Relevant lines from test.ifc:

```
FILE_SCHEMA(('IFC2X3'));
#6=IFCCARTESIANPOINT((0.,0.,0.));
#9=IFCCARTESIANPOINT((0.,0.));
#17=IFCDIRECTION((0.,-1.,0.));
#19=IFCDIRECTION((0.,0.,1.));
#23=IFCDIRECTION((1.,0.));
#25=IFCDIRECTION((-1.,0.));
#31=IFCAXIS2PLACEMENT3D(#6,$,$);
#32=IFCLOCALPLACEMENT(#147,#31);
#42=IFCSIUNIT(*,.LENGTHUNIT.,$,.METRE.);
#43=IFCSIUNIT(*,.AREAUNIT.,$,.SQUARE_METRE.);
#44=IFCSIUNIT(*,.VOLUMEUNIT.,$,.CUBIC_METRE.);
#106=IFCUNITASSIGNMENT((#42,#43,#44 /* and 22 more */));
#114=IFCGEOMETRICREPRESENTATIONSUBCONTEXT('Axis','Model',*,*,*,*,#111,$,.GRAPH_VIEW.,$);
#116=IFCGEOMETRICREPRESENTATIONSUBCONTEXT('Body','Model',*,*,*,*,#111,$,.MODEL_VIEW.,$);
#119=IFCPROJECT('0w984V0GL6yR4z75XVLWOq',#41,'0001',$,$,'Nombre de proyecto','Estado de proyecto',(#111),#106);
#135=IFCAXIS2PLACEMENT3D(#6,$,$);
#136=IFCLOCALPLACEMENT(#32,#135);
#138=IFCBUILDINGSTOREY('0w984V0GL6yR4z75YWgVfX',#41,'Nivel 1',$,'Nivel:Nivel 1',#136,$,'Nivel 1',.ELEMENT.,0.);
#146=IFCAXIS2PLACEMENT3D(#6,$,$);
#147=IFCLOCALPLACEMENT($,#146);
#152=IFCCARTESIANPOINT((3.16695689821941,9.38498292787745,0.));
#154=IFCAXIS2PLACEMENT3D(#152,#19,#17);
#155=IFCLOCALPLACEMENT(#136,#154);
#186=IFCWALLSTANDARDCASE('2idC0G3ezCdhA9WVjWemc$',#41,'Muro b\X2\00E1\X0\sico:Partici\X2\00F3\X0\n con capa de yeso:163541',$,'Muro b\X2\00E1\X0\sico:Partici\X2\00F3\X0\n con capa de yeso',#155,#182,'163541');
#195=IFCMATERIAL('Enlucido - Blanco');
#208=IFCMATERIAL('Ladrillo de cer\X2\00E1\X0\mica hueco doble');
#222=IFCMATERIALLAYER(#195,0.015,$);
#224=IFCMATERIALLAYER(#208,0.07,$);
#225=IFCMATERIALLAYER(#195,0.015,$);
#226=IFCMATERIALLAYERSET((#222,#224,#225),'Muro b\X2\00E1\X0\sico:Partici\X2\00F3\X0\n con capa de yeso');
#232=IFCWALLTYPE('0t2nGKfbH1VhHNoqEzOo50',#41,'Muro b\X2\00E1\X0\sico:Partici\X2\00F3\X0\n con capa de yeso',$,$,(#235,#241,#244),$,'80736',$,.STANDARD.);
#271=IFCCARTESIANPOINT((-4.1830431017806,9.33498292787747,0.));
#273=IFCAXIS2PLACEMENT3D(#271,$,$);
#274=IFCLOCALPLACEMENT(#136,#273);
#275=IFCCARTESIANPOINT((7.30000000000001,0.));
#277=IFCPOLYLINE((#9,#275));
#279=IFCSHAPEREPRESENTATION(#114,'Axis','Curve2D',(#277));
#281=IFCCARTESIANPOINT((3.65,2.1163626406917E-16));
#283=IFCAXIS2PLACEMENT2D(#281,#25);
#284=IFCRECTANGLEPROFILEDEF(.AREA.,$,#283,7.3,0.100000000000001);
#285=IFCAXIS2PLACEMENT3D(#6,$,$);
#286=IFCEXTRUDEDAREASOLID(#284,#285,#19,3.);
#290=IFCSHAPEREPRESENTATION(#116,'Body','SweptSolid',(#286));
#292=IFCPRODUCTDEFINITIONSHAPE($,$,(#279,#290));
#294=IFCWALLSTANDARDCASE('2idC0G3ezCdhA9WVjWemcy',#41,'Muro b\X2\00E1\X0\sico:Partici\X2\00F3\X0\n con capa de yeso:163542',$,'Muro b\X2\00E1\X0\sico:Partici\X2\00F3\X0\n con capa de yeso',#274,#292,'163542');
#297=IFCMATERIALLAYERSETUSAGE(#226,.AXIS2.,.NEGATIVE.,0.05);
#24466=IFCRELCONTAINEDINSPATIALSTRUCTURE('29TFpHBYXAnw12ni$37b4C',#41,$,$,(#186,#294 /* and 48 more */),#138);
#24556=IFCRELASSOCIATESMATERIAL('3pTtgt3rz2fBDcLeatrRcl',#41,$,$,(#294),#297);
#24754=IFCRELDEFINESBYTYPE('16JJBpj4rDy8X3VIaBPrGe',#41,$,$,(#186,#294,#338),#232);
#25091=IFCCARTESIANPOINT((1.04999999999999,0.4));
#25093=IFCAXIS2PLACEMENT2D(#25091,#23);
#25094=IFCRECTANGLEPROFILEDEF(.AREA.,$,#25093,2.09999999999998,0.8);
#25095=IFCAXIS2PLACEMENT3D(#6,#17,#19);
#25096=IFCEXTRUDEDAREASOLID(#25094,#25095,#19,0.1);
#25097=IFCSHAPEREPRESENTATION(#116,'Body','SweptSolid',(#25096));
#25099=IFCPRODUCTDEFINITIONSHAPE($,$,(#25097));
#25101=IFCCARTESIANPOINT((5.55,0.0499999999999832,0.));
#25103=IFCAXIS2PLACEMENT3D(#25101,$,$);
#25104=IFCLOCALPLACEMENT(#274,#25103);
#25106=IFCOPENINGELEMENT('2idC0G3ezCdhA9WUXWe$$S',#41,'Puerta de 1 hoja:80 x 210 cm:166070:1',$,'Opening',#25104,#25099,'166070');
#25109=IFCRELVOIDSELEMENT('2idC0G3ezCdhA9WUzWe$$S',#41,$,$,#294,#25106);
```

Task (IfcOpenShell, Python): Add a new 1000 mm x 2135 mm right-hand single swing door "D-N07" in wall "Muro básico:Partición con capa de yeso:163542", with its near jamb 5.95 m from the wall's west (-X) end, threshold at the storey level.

```python
import numpy as np
import ifcopenshell
import ifcopenshell.api.feature
import ifcopenshell.api.geometry
import ifcopenshell.api.root
import ifcopenshell.api.spatial
import ifcopenshell.api.type
import ifcopenshell.geom
import ifcopenshell.util.element
import ifcopenshell.util.placement
import ifcopenshell.util.representation
import ifcopenshell.util.shape
import ifcopenshell.util.unit

model = ifcopenshell.open("test.ifc")
unit_scale = ifcopenshell.util.unit.calculate_unit_scale(model)
settings = ifcopenshell.geom.settings()


def volume(element):
    """Net volume in cubic metres, openings subtracted."""
    shape = ifcopenshell.geom.create_shape(settings, element)
    return ifcopenshell.util.shape.get_volume(shape.geometry)


wall = model.by_guid("2idC0G3ezCdhA9WVjWemcy")
storey = ifcopenshell.util.element.get_container(wall, ifc_class="IfcBuildingStorey")
context = ifcopenshell.util.representation.get_context(model, "Model", "Body", "MODEL_VIEW")
before = volume(wall)

width, height, from_end, sill = 1, 2.135, 5.95, 0.0  # metres

# The wall runs along its own X axis, and the end named is its -X end.
wall_shape = ifcopenshell.geom.create_shape(settings, wall)
x, y, z = ifcopenshell.util.shape.get_vertices(wall_shape.geometry).T
start = x.min() + from_end
face, thickness = float(y.min()), float(y.max() - y.min())
wall_matrix = ifcopenshell.util.placement.get_local_placement(wall.ObjectPlacement)
level = ifcopenshell.util.placement.get_local_placement(storey.ObjectPlacement)[2, 3]


def in_wall(x, y):
    """Placement at x, y metres in the wall's axes, at sill height."""
    matrix = wall_matrix.copy()
    matrix[:, 3] = wall_matrix @ np.array([x / unit_scale, y / unit_scale, 0.0, 1.0])
    matrix[2, 3] = level + sill / unit_scale
    return matrix


# Opening: a box that overshoots both wall faces by 50 mm.
opening = ifcopenshell.api.root.create_entity(model, ifc_class="IfcOpeningElement")
box = ifcopenshell.api.geometry.add_wall_representation(
    model, context=context, length=width, height=height, thickness=thickness + 0.1
)
ifcopenshell.api.geometry.assign_representation(model, product=opening, representation=box)
ifcopenshell.api.geometry.edit_object_placement(model, product=opening, matrix=in_wall(start, face - 0.05), is_si=False)
ifcopenshell.api.feature.add_feature(model, feature=opening, element=wall)

door = ifcopenshell.api.root.create_entity(model, ifc_class="IfcDoor", name="D-N07")
door.OverallWidth, door.OverallHeight = width / unit_scale, height / unit_scale
body = ifcopenshell.api.geometry.add_door_representation(
    model,
    context=context,
    overall_width=door.OverallWidth,
    overall_height=door.OverallHeight,
    operation_type="SINGLE_SWING_RIGHT",
    lining_properties={"LiningDepth": thickness / unit_scale, "ThresholdDepth": thickness / unit_scale},
)
ifcopenshell.api.geometry.assign_representation(model, product=door, representation=body)
ifcopenshell.api.spatial.assign_container(model, products=[door], relating_structure=storey)
fills = ifcopenshell.api.feature.add_filling(model, opening=opening, element=door)
fills.OwnerHistory = door.OwnerHistory  # required in IFC2X3

# IFC2X3 keeps the operation on the door style.
style = ifcopenshell.api.root.create_entity(model, ifc_class="IfcDoorStyle", name="D-N07")
style.OperationType, style.ConstructionType = "SINGLE_SWING_RIGHT", "NOTDEFINED"
style.ParameterTakesPrecedence = style.Sizeable = False
ifcopenshell.api.type.assign_type(model, related_objects=[door], relating_type=style)

# The lining spans the wall, so the door starts at the wall face.
ifcopenshell.api.geometry.edit_object_placement(model, product=door, matrix=in_wall(start, face), is_si=False)

after = volume(wall)

print(f"wall volume {before:.3f} -> {after:.3f} m3")

model.write("test_edited.ifc")
```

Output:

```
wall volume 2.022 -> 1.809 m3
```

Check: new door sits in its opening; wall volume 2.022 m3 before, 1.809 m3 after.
